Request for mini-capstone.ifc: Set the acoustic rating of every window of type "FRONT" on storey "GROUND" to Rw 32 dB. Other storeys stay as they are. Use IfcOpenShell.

First a look at what the model holds.

```python
import ifcopenshell
import ifcopenshell.util.element

model = ifcopenshell.open("mini-capstone.ifc")
print(model.schema)
storey = next(s for s in model.by_type("IfcBuildingStorey") if s.Name == "GROUND")
windows = [e for e in ifcopenshell.util.element.get_decomposition(storey) if e.is_a("IfcWindow")]
seen = {}
for e in windows:
    element_type = ifcopenshell.util.element.get_type(e)
    key = (element_type.Name if element_type != e and element_type else None, ifcopenshell.util.element.get_pset(e, "Pset_WindowCommon", "AcousticRating"))
    seen[key] = seen.get(key, 0) + 1
for (name, value), count in sorted(seen.items(), key=str):
    print(count, "x", name, "|", value)
```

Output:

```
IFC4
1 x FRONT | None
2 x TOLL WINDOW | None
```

```python
import ifcopenshell
import ifcopenshell.api.pset
import ifcopenshell.util.element

model = ifcopenshell.open("mini-capstone.ifc")

storey = next(s for s in model.by_type("IfcBuildingStorey") if s.Name == "GROUND")
windows = [e for e in ifcopenshell.util.element.get_decomposition(storey) if e.is_a("IfcWindow")]

count = 0
for e in windows:
    element_type = ifcopenshell.util.element.get_type(e)
    if element_type in (None, e) or element_type.Name != "FRONT":
        continue
    # add_pset returns the element's existing set when there is one.
    pset = ifcopenshell.api.pset.add_pset(model, product=e, name="Pset_WindowCommon")
    ifcopenshell.api.pset.edit_pset(model, pset=pset, properties={"AcousticRating": "Rw 32 dB"})
    count += 1

print(count, "windows updated")

model.write("mini-capstone_v2.ifc")
```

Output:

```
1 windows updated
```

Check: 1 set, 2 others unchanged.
